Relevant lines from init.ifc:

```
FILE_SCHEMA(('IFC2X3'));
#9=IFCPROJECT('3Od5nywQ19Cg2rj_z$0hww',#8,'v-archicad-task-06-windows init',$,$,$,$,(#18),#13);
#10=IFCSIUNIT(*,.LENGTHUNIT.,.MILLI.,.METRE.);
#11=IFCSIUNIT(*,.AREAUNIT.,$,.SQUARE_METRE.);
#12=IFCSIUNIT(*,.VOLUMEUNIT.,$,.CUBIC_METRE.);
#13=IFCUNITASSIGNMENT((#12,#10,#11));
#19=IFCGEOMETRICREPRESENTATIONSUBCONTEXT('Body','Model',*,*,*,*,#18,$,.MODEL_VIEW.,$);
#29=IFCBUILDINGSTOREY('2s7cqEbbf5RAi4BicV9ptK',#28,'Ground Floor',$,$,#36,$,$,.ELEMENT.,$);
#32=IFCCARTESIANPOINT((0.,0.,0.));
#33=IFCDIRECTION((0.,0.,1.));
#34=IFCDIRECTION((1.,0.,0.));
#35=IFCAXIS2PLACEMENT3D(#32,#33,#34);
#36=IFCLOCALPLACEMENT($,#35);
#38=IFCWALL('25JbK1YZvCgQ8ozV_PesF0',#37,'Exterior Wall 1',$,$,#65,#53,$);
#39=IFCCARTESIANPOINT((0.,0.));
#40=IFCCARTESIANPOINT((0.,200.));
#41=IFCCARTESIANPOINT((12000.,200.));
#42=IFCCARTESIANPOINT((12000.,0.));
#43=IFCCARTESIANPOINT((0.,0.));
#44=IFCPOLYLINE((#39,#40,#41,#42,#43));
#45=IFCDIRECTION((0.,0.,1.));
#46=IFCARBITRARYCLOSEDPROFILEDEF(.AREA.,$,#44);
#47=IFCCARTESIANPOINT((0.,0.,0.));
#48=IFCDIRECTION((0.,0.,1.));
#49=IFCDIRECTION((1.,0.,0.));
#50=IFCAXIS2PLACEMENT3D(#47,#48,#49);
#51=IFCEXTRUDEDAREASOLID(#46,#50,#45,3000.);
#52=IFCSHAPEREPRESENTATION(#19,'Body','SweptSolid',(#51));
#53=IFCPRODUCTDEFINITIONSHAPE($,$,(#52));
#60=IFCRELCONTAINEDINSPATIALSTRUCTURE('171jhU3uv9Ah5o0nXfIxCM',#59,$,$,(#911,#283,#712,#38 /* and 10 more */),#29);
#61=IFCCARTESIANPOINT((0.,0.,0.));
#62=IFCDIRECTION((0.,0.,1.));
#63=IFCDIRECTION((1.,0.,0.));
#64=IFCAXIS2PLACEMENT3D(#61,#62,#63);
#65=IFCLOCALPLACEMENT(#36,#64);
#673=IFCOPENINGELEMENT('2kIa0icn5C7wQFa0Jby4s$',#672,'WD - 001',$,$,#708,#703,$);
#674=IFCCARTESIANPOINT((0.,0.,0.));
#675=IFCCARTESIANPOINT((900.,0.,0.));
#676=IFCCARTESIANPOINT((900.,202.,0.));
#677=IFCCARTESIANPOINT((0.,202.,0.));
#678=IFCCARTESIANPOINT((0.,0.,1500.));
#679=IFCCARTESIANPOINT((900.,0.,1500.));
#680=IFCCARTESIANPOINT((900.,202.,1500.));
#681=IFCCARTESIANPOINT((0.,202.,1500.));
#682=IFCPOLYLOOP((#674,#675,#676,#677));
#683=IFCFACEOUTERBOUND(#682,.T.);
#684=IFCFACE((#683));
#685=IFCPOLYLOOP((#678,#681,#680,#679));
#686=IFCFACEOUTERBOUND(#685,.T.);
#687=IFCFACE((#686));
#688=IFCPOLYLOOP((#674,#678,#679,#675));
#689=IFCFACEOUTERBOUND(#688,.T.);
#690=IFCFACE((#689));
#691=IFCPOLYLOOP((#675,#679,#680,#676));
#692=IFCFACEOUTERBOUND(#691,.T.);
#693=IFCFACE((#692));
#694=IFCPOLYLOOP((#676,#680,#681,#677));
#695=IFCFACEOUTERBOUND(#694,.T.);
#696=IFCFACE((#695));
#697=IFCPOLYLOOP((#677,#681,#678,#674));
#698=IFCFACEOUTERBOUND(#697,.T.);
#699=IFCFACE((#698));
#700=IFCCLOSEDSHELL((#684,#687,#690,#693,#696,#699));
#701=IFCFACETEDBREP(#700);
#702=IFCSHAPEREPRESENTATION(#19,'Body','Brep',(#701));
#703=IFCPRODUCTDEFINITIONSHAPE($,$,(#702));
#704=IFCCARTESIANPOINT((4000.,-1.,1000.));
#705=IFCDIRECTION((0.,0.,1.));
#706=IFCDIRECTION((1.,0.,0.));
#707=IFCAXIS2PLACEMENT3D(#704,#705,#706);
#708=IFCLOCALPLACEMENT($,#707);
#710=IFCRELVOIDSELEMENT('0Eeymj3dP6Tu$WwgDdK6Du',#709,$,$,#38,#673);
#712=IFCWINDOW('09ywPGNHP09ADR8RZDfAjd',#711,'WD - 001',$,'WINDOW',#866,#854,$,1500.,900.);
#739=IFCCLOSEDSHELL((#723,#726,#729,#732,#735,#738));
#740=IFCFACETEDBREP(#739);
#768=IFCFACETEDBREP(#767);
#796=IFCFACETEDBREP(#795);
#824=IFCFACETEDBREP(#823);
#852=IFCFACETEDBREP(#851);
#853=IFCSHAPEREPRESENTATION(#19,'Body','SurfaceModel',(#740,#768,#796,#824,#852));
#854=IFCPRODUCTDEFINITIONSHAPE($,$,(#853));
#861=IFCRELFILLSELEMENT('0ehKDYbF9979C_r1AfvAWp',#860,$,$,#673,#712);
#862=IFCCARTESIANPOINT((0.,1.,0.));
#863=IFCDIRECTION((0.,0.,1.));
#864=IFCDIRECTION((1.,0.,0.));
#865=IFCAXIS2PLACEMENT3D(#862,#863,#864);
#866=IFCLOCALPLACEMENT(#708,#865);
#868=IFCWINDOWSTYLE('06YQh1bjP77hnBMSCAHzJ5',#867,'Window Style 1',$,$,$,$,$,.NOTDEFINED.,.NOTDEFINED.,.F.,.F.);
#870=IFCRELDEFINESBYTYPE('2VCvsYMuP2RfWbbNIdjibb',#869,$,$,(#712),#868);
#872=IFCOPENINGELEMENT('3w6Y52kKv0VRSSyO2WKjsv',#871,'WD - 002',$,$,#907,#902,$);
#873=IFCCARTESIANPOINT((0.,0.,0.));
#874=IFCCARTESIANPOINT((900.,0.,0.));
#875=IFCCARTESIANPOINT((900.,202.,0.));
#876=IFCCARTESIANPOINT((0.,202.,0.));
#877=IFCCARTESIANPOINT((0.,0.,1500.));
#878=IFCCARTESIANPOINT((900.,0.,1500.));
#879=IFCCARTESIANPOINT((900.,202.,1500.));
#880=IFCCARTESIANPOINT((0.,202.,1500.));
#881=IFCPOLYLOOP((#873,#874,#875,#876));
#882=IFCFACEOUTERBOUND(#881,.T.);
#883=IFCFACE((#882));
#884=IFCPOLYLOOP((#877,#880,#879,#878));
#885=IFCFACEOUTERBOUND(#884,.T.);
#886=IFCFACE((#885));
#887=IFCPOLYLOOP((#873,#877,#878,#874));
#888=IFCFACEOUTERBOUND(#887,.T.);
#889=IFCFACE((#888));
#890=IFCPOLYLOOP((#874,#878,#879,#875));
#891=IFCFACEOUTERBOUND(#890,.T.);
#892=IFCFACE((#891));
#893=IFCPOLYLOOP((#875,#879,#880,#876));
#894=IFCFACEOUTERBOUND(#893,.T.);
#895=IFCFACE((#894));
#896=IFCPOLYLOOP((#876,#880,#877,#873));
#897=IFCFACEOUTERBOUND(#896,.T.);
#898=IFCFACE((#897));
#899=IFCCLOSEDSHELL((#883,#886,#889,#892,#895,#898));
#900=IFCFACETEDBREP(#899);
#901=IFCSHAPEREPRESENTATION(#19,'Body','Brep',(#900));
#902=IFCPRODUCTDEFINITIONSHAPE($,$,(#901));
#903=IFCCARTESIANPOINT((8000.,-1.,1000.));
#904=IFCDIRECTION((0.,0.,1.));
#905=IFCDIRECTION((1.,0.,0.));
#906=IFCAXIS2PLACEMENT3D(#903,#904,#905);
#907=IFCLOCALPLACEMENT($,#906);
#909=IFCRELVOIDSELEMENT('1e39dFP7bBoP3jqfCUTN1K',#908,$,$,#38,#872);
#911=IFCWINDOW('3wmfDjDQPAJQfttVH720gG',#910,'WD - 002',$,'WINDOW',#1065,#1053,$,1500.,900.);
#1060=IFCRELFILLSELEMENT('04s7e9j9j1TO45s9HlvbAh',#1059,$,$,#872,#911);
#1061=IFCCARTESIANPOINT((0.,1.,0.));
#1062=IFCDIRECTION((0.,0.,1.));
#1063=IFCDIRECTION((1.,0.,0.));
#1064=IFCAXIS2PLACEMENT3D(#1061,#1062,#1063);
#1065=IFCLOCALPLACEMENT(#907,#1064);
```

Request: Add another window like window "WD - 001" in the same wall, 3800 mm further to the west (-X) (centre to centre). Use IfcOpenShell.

```python
import ifcopenshell
import ifcopenshell.api.feature
import ifcopenshell.api.geometry
import ifcopenshell.api.root
import ifcopenshell.geom
import ifcopenshell.util.element
import ifcopenshell.util.placement
import ifcopenshell.util.shape
import ifcopenshell.util.unit

model = ifcopenshell.open("init.ifc")
unit_scale = ifcopenshell.util.unit.calculate_unit_scale(model)
settings = ifcopenshell.geom.settings()


def volume(element):
    """Net volume in cubic metres, openings subtracted."""
    shape = ifcopenshell.geom.create_shape(settings, element)
    return ifcopenshell.util.shape.get_volume(shape.geometry)


window = model.by_guid("09ywPGNHP09ADR8RZDfAjd")
opening = window.FillsVoids[0].RelatingOpeningElement
wall = opening.VoidsElements[0].RelatingBuildingElement
before = volume(wall)
shift = ifcopenshell.util.placement.get_local_placement(wall.ObjectPlacement)[:3, 0] * -3.8 / unit_scale

# copy_class copies the void relationship, type, container and properties, but no geometry.
new_opening = ifcopenshell.api.root.copy_class(model, product=opening)
new_opening.Representation = ifcopenshell.util.element.copy_deep(
    model, opening.Representation, exclude=["IfcGeometricRepresentationContext", "IfcRepresentationMap"]
)
new_window = ifcopenshell.api.root.copy_class(model, product=window)
new_window.Representation = ifcopenshell.util.element.copy_deep(
    model, window.Representation, exclude=["IfcGeometricRepresentationContext", "IfcRepresentationMap"]
)
fills = ifcopenshell.api.feature.add_filling(model, opening=new_opening, element=new_window)
fills.OwnerHistory = new_window.OwnerHistory  # required in IFC2X3

for old, new in ((opening, new_opening), (window, new_window)):
    matrix = ifcopenshell.util.placement.get_local_placement(old.ObjectPlacement)
    matrix[:3, 3] += shift
    ifcopenshell.api.geometry.edit_object_placement(model, product=new, matrix=matrix, is_si=False)

after = volume(wall)

print(f"wall volume {before:.3f} -> {after:.3f} m3")

model.write("init-out.ifc")
```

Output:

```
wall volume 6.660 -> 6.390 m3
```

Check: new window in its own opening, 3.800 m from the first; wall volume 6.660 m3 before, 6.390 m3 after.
